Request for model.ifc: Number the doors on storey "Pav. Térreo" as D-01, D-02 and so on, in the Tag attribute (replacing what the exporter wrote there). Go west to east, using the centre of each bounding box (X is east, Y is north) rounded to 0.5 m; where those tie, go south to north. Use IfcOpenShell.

First a look at what the model holds.

```python
import ifcopenshell
import ifcopenshell.util.element
import ifcopenshell.util.placement

model = ifcopenshell.open("model.ifc")
print(model.schema)
storey = next(s for s in model.by_type("IfcBuildingStorey") if s.Name == "Pav. Térreo")
doors = [e for e in ifcopenshell.util.element.get_decomposition(storey) if e.is_a("IfcDoor")]
for e in sorted(doors, key=lambda e: e.id()):
    origin = ifcopenshell.util.placement.get_local_placement(e.ObjectPlacement)[:3, 3]
    print(e.id(), e.Tag, e.Name, origin.round(2) + 0.0, sep=" | ")
```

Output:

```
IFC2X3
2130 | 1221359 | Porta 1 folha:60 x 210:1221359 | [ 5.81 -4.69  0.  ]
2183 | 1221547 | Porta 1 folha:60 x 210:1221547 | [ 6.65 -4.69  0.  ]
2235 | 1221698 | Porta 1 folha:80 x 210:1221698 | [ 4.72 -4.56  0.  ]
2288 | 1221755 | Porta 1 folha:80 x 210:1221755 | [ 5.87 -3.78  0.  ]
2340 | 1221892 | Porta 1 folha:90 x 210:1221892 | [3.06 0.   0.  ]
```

```python
import ifcopenshell
import ifcopenshell.geom
import ifcopenshell.util.element
import ifcopenshell.util.shape

model = ifcopenshell.open("model.ifc")
settings = ifcopenshell.geom.settings()
settings.set("use-world-coords", True)


def centre(element):
    shape = ifcopenshell.geom.create_shape(settings, element)
    return ifcopenshell.util.shape.get_bbox_centroid(shape.geometry)


storey = next(s for s in model.by_type("IfcBuildingStorey") if s.Name == "Pav. Térreo")
doors = [e for e in ifcopenshell.util.element.get_decomposition(storey) if e.is_a("IfcDoor")]

# Insertion points can sit at a corner or the storey origin, so sort by the geometry (in metres).
centres = {e: centre(e) for e in doors}
doors.sort(key=lambda e: (round(centres[e][0] / 0.5), centres[e][1]))

for i, e in enumerate(doors, start=1):
    number = f"D-{i:02d}"
    e.Tag = number
    print(e.id(), number)

model.write("model_updated.ifc")
```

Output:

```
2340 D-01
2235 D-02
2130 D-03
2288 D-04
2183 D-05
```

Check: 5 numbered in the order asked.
